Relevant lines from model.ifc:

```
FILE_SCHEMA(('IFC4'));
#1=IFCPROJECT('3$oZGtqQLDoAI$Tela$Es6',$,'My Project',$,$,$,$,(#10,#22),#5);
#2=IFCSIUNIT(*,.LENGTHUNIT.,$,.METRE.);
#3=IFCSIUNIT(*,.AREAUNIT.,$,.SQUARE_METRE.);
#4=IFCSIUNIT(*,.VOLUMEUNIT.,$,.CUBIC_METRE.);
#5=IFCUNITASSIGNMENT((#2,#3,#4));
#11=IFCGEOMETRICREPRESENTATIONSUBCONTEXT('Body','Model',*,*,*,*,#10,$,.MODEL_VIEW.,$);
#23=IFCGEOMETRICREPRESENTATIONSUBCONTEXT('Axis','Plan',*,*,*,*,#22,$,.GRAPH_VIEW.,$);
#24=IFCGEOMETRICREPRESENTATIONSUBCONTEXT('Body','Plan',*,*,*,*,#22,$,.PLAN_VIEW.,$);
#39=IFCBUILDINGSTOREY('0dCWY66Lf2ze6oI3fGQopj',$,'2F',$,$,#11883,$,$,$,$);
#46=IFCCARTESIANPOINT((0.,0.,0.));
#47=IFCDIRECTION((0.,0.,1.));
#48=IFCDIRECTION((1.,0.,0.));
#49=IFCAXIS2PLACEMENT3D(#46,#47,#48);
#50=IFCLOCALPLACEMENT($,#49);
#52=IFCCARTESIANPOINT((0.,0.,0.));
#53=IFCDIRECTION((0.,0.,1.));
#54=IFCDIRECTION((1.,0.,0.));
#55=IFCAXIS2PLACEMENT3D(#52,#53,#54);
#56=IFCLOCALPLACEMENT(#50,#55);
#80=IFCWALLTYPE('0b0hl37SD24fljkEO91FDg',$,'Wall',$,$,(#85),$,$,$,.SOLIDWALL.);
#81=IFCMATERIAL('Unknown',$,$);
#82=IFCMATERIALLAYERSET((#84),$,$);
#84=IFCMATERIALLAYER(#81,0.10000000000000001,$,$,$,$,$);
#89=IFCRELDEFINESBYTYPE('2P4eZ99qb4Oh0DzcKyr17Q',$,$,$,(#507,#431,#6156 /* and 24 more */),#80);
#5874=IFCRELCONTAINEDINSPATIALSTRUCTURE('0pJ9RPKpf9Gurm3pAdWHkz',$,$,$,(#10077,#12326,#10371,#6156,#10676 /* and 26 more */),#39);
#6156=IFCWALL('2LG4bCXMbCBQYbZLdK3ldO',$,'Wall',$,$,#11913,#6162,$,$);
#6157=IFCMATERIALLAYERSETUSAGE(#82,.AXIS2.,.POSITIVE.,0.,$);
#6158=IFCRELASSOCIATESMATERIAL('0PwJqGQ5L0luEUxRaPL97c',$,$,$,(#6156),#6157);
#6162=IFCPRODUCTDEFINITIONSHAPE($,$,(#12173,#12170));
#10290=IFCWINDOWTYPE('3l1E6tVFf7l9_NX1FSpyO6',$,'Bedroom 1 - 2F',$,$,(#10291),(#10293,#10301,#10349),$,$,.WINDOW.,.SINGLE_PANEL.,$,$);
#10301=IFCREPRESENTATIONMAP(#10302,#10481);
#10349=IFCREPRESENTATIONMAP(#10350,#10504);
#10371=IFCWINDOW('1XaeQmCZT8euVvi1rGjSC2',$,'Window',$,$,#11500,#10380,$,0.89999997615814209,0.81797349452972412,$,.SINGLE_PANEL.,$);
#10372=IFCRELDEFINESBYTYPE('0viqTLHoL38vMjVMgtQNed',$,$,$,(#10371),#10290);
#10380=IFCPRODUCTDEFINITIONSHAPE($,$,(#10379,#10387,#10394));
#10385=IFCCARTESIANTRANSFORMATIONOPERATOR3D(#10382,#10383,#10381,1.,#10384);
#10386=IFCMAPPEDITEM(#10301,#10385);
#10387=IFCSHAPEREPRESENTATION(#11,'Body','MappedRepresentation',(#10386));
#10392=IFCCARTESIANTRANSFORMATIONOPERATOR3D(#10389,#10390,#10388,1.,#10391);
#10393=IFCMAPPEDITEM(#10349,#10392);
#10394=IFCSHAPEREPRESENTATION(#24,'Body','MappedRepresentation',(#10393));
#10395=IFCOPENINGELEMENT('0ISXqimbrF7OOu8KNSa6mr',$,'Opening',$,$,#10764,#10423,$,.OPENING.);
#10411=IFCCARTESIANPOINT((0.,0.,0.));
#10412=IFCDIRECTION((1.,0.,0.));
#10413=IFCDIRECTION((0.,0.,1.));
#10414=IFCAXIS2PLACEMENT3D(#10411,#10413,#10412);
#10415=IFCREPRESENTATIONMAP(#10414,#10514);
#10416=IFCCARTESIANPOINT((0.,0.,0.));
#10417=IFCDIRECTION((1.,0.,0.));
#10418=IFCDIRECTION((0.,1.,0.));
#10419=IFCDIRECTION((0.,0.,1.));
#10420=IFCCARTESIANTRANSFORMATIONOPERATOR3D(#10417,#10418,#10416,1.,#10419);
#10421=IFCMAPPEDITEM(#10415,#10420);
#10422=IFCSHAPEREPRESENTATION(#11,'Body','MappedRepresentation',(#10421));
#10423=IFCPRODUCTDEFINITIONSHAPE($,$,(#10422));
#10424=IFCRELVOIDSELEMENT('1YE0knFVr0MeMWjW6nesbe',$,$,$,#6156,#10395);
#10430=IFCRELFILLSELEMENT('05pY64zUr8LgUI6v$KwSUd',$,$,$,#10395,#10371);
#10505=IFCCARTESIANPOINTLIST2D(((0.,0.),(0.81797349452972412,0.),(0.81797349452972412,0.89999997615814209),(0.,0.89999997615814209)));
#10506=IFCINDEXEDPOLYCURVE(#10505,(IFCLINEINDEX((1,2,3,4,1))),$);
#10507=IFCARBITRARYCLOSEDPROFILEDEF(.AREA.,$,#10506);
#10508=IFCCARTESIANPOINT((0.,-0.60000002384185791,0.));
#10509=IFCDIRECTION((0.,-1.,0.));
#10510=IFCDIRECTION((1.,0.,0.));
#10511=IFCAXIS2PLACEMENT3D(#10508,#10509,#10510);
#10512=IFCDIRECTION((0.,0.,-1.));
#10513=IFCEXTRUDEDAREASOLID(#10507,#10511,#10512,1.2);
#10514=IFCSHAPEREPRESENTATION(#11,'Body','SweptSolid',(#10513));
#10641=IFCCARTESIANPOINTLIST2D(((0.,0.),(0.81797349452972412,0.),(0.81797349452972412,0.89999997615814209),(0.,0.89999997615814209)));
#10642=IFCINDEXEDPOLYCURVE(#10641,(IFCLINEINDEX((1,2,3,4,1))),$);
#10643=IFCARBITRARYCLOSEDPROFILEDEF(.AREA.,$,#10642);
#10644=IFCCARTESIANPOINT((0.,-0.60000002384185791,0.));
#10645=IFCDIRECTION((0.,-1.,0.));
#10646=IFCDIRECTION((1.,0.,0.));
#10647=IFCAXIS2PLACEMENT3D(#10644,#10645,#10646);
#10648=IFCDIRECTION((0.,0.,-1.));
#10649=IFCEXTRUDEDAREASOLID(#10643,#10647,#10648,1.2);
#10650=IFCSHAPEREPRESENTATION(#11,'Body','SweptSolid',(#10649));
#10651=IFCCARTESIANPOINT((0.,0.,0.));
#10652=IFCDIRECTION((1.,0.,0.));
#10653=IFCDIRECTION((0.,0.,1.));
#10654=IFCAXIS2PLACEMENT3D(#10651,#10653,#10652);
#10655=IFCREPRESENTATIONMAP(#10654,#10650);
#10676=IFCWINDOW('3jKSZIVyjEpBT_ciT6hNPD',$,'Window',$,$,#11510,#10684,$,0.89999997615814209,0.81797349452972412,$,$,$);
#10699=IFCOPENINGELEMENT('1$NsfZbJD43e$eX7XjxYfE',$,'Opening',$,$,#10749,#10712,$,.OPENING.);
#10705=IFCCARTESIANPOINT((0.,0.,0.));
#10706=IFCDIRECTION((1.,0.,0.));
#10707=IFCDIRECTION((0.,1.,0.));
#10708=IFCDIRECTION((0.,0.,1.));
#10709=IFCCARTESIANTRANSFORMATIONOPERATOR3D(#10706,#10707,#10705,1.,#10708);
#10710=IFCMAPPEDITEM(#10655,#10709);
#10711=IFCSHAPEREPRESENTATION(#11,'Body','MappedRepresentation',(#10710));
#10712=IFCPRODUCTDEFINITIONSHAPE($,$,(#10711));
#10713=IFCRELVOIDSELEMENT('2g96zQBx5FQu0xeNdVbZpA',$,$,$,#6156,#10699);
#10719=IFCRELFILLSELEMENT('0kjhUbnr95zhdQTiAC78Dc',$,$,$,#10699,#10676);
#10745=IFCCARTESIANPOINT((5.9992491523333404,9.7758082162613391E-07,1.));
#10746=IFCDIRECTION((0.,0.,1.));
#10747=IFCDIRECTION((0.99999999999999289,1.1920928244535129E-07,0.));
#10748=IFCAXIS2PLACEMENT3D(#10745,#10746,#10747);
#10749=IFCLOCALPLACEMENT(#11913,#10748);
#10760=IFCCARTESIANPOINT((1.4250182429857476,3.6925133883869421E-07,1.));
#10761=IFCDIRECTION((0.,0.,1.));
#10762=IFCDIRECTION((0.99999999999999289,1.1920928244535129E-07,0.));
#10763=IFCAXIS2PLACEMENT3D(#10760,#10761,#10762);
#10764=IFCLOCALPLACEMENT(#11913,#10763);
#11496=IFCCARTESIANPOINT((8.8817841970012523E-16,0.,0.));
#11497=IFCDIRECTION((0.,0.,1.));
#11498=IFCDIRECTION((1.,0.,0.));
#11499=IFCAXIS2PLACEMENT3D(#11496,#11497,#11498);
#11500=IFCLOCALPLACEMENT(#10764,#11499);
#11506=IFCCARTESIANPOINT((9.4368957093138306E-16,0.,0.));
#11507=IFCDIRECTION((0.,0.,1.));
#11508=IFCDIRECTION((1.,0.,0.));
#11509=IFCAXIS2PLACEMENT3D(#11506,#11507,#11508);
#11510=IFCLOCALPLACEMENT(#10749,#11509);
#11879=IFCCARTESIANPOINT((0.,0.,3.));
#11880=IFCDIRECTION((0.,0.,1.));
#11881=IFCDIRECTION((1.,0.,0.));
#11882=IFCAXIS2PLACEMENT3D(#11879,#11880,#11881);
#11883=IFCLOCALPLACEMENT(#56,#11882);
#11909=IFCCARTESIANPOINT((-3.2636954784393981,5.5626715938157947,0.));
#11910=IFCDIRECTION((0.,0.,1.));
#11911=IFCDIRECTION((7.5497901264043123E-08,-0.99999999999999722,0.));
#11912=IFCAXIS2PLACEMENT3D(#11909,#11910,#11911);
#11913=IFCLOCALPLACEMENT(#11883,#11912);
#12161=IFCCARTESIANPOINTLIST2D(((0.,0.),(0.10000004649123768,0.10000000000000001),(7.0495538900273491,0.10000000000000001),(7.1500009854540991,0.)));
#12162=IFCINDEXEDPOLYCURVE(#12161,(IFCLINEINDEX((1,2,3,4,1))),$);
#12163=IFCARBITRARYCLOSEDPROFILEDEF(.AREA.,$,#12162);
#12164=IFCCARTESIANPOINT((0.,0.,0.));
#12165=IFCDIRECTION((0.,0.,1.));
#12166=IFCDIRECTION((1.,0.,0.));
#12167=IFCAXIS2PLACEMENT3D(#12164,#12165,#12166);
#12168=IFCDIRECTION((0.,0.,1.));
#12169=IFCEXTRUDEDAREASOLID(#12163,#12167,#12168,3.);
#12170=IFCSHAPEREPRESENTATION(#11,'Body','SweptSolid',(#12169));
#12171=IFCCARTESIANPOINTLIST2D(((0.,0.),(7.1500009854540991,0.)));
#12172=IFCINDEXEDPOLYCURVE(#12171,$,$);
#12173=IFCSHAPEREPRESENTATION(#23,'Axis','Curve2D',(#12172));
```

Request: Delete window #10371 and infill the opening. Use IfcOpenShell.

```python
import ifcopenshell
import ifcopenshell.api.feature
import ifcopenshell.api.root
import ifcopenshell.geom
import ifcopenshell.util.shape

model = ifcopenshell.open("model.ifc")
settings = ifcopenshell.geom.settings()


def volume(element):
    """Net volume in cubic metres, openings subtracted."""
    shape = ifcopenshell.geom.create_shape(settings, element)
    return ifcopenshell.util.shape.get_volume(shape.geometry)


window = model.by_guid("1XaeQmCZT8euVvi1rGjSC2")
opening = window.FillsVoids[0].RelatingOpeningElement
wall = opening.VoidsElements[0].RelatingBuildingElement
before = volume(wall)

ifcopenshell.api.root.remove_product(model, product=window)
ifcopenshell.api.feature.remove_feature(model, feature=opening)

after = volume(wall)

print(f"wall volume {before:.3f} -> {after:.3f} m3")

model.write("model_updated.ifc")
```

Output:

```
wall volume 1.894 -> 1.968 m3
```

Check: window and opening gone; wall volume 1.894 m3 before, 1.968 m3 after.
